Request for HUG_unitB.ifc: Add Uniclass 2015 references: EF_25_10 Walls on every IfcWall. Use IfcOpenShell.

First a look at what the model holds.

```python
import ifcopenshell

model = ifcopenshell.open("HUG_unitB.ifc")
print(model.schema)
print("classifications:", [c.Name for c in model.by_type("IfcClassification")])
for ifc_class in ("IfcDoor", "IfcRoof", "IfcStair", "IfcWall", "IfcWindow"):
    print(ifc_class, len(model.by_type(ifc_class)))
```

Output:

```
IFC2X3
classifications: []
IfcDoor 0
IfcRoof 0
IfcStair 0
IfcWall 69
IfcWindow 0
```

```python
import ifcopenshell
import ifcopenshell.api.classification

model = ifcopenshell.open("HUG_unitB.ifc")

# IFC2X3 requires Source and Edition and has no link from the project to the system.
system = model.create_entity("IfcClassification", Source="NBS", Edition="2015", Name="Uniclass 2015")

codes = {
    "IfcWall": ("EF_25_10", "Walls"),
}
for ifc_class, (code, name) in codes.items():
    products = model.by_type(ifc_class)
    ifcopenshell.api.classification.add_reference(
        model, products=products, classification=system, identification=code, name=name
    )
    print(code, len(products))

model.write("HUG_unitB_rev.ifc")
```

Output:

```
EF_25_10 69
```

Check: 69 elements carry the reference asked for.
